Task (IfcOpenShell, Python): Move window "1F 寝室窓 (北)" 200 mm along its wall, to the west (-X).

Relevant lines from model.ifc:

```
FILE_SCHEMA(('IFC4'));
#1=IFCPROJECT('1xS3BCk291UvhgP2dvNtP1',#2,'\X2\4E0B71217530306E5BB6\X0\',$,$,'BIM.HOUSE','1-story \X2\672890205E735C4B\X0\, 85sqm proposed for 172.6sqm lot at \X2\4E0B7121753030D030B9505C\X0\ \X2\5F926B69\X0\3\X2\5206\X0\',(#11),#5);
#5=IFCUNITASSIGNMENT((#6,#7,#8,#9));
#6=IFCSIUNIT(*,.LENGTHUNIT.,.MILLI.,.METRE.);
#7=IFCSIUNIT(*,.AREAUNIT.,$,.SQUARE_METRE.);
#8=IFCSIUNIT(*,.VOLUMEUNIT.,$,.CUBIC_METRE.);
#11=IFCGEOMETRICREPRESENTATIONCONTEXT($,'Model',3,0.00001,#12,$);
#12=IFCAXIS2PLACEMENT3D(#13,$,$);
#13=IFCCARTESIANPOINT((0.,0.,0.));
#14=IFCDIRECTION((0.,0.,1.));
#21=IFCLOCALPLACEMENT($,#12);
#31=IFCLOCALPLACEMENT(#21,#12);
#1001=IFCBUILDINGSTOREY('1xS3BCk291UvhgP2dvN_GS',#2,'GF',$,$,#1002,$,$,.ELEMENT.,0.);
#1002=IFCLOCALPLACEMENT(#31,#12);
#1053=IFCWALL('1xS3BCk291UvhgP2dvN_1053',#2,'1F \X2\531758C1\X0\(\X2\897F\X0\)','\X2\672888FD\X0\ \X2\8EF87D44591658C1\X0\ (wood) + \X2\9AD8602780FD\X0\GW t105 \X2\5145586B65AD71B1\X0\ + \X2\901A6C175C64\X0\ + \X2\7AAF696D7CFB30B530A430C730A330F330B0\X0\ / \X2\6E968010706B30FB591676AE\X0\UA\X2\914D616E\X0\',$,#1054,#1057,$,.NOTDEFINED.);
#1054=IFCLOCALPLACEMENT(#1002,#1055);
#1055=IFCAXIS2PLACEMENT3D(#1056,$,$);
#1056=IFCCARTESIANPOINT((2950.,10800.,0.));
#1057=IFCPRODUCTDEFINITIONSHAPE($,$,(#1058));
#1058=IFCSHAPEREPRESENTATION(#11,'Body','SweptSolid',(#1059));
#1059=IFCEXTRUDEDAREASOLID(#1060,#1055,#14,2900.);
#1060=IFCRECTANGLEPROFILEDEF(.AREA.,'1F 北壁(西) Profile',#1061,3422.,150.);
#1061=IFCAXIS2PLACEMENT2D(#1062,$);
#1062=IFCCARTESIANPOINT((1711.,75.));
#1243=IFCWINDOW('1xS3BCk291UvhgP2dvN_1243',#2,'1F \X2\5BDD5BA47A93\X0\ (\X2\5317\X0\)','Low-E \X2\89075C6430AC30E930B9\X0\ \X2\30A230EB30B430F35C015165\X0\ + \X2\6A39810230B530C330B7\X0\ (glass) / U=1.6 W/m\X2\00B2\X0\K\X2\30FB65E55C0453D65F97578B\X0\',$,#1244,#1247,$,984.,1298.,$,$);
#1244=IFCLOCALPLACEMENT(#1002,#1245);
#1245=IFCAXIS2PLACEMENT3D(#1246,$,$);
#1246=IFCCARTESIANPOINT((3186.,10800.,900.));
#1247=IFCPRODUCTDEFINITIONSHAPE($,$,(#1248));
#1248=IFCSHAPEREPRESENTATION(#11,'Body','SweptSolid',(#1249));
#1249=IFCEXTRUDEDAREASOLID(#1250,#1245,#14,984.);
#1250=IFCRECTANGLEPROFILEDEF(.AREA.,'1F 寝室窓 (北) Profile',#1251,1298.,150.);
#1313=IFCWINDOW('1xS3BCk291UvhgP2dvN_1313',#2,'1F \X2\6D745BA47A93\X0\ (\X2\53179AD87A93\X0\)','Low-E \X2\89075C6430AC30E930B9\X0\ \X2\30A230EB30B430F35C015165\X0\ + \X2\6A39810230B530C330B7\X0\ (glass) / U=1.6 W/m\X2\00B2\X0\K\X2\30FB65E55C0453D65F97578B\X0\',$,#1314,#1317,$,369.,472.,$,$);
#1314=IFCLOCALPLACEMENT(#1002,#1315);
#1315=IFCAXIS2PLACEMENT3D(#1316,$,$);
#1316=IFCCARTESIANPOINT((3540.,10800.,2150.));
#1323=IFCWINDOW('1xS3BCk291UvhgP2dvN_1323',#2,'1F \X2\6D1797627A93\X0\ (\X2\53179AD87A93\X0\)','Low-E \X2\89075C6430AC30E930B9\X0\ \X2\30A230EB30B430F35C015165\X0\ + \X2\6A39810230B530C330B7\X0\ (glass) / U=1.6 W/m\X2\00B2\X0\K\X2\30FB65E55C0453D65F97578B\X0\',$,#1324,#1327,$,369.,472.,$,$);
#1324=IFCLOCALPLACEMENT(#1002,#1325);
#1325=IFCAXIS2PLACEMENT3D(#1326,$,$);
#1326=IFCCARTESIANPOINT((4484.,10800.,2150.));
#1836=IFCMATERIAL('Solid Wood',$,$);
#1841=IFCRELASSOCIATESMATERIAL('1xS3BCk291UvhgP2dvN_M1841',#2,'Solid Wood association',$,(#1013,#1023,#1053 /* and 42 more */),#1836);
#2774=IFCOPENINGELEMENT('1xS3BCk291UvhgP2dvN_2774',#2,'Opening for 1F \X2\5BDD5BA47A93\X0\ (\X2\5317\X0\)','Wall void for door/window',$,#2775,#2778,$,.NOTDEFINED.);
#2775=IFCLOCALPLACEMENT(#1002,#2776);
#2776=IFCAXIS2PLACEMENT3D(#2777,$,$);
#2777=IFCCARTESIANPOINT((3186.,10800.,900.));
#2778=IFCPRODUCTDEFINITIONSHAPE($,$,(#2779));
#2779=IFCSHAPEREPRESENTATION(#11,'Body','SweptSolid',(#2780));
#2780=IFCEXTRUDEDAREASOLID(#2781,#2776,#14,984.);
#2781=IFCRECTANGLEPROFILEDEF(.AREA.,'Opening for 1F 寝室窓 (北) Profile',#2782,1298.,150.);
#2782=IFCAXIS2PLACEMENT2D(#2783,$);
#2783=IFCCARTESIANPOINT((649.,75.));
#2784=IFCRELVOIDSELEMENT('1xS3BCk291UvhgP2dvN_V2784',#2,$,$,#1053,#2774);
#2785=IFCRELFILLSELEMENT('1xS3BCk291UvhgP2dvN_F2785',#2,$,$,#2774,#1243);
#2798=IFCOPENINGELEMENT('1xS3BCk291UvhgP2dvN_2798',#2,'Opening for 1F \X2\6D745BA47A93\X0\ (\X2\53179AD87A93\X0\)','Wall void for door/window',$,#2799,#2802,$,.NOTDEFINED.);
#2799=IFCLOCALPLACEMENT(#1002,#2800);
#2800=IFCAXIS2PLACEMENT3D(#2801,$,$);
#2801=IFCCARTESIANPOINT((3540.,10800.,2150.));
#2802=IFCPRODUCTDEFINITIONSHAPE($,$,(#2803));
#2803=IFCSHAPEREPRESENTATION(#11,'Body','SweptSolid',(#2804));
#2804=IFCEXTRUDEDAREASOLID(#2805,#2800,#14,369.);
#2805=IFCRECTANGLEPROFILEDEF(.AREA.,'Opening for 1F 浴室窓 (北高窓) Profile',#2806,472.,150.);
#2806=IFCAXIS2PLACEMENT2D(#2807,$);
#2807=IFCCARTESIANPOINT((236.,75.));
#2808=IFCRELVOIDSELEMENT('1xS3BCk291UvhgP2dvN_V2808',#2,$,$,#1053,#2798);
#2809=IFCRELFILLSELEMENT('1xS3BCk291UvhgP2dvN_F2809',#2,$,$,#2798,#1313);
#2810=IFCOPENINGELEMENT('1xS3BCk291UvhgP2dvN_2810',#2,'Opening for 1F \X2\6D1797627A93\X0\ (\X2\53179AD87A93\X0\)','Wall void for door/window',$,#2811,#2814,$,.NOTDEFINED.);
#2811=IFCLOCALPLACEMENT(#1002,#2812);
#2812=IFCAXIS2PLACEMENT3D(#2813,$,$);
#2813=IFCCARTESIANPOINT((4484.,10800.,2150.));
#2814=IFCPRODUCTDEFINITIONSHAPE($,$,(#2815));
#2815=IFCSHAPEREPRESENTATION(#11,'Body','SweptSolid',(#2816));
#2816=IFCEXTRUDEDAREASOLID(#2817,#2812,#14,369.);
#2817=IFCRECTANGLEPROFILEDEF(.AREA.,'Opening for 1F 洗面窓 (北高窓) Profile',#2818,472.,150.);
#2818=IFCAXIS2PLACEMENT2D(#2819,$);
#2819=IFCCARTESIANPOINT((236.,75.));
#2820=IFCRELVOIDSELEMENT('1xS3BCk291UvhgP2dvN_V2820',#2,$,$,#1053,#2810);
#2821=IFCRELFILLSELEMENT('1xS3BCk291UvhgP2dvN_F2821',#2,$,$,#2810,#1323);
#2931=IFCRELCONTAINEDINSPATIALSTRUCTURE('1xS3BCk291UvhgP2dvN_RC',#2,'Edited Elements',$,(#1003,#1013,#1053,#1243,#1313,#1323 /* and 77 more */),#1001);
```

```python
import ifcopenshell
import ifcopenshell.api.geometry
import ifcopenshell.util.placement
import ifcopenshell.util.unit

model = ifcopenshell.open("model.ifc")
unit_scale = ifcopenshell.util.unit.calculate_unit_scale(model)

window = model.by_guid("1xS3BCk291UvhgP2dvN_1243")
opening = window.FillsVoids[0].RelatingOpeningElement
wall = opening.VoidsElements[0].RelatingBuildingElement

wall_matrix = ifcopenshell.util.placement.get_local_placement(wall.ObjectPlacement)
shift = wall_matrix[:3, 0] * -0.2 / unit_scale
before = ifcopenshell.util.placement.get_local_placement(window.ObjectPlacement)[:3, 3].copy()

# The window is not placed relative to its opening, so move both.
for product in (opening, window):
    matrix = ifcopenshell.util.placement.get_local_placement(product.ObjectPlacement)
    matrix[:3, 3] += shift
    ifcopenshell.api.geometry.edit_object_placement(model, product=product, matrix=matrix, is_si=False)

after = ifcopenshell.util.placement.get_local_placement(window.ObjectPlacement)[:3, 3]
print("window moved by", (after - before).round(3) + 0.0)

model.write("model_v2.ifc")
```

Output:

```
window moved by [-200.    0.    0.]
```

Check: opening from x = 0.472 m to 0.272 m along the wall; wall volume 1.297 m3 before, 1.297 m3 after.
